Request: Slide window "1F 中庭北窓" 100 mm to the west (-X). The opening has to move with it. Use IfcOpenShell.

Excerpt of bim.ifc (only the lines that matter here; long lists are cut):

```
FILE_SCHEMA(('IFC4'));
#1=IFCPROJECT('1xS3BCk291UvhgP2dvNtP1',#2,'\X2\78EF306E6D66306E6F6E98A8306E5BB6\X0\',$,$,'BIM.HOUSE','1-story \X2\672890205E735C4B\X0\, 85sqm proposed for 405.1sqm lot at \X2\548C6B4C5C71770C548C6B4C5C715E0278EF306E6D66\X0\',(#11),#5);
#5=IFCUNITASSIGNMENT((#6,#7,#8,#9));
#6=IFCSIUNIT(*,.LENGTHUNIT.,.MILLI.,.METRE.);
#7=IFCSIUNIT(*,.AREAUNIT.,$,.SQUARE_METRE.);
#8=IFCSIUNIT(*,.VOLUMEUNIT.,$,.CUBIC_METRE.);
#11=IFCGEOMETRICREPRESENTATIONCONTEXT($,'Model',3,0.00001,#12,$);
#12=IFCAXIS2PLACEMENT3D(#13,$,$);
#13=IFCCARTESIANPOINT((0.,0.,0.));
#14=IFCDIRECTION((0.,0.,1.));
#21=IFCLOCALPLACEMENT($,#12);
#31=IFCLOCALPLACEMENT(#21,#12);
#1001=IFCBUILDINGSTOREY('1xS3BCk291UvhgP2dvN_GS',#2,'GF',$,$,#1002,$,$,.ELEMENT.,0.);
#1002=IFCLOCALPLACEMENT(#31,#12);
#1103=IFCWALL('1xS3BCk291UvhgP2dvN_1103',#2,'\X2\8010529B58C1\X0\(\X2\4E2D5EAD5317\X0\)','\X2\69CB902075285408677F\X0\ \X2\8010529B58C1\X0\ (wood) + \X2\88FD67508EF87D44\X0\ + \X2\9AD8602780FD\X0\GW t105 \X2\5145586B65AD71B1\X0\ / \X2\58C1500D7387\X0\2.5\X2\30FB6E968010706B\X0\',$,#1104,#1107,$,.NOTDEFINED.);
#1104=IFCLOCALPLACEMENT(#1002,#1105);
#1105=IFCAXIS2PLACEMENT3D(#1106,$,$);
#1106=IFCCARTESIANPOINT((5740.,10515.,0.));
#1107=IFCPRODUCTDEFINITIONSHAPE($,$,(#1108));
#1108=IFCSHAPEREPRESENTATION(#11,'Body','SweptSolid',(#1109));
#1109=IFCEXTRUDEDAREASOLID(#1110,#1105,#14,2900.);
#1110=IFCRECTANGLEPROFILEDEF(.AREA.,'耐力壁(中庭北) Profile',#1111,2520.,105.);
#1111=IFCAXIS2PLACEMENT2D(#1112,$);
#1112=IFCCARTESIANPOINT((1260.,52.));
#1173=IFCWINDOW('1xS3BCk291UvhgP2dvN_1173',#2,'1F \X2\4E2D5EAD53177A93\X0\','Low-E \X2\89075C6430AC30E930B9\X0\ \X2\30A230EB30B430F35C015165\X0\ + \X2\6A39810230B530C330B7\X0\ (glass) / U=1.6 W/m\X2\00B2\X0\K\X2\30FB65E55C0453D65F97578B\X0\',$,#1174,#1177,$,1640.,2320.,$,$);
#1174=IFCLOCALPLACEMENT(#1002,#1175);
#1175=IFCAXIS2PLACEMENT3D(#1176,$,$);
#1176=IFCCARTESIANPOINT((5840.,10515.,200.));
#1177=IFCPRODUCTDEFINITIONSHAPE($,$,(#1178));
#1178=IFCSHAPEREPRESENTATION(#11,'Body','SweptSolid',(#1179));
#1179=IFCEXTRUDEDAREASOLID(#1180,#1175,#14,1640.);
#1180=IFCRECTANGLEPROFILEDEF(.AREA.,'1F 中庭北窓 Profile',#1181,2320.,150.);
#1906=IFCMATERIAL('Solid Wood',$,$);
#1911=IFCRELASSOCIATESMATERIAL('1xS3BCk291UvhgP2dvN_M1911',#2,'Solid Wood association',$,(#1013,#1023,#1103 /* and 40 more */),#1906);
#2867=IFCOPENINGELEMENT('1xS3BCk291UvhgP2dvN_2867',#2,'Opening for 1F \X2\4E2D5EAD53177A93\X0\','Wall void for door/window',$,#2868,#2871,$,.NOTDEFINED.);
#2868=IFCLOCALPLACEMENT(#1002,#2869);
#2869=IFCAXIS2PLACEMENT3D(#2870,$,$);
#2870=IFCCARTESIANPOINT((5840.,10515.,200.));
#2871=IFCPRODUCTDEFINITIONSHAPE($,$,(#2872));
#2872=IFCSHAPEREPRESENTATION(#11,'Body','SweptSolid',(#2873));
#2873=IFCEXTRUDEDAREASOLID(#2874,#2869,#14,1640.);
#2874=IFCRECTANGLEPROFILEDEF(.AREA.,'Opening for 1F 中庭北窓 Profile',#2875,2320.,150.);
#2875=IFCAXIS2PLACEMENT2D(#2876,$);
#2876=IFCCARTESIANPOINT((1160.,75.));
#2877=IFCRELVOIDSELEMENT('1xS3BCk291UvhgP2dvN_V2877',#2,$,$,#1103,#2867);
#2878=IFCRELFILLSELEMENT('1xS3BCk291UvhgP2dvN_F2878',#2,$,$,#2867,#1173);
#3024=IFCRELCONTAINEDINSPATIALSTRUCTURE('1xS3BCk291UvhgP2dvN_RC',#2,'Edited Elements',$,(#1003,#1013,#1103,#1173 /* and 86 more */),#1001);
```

```python
import ifcopenshell
import ifcopenshell.api.geometry
import ifcopenshell.util.placement

model = ifcopenshell.open("bim.ifc")

window = model.by_guid("1xS3BCk291UvhgP2dvN_1173")
opening = window.FillsVoids[0].RelatingOpeningElement
wall = opening.VoidsElements[0].RelatingBuildingElement

wall_matrix = ifcopenshell.util.placement.get_local_placement(wall.ObjectPlacement)
shift = wall_matrix[:3, 0] * -100.0
before = ifcopenshell.util.placement.get_local_placement(window.ObjectPlacement)[:3, 3].copy()

# The window is not placed relative to its opening, so move both.
for product in (opening, window):
    matrix = ifcopenshell.util.placement.get_local_placement(product.ObjectPlacement)
    matrix[:3, 3] += shift
    ifcopenshell.api.geometry.edit_object_placement(model, product=product, matrix=matrix, is_si=False)

after = ifcopenshell.util.placement.get_local_placement(window.ObjectPlacement)[:3, 3]
print("window moved by", (after - before).round(3) + 0.0)

model.write("bim_v2.ifc")
```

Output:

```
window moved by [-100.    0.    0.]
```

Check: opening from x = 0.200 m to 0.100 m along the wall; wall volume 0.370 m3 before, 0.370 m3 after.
